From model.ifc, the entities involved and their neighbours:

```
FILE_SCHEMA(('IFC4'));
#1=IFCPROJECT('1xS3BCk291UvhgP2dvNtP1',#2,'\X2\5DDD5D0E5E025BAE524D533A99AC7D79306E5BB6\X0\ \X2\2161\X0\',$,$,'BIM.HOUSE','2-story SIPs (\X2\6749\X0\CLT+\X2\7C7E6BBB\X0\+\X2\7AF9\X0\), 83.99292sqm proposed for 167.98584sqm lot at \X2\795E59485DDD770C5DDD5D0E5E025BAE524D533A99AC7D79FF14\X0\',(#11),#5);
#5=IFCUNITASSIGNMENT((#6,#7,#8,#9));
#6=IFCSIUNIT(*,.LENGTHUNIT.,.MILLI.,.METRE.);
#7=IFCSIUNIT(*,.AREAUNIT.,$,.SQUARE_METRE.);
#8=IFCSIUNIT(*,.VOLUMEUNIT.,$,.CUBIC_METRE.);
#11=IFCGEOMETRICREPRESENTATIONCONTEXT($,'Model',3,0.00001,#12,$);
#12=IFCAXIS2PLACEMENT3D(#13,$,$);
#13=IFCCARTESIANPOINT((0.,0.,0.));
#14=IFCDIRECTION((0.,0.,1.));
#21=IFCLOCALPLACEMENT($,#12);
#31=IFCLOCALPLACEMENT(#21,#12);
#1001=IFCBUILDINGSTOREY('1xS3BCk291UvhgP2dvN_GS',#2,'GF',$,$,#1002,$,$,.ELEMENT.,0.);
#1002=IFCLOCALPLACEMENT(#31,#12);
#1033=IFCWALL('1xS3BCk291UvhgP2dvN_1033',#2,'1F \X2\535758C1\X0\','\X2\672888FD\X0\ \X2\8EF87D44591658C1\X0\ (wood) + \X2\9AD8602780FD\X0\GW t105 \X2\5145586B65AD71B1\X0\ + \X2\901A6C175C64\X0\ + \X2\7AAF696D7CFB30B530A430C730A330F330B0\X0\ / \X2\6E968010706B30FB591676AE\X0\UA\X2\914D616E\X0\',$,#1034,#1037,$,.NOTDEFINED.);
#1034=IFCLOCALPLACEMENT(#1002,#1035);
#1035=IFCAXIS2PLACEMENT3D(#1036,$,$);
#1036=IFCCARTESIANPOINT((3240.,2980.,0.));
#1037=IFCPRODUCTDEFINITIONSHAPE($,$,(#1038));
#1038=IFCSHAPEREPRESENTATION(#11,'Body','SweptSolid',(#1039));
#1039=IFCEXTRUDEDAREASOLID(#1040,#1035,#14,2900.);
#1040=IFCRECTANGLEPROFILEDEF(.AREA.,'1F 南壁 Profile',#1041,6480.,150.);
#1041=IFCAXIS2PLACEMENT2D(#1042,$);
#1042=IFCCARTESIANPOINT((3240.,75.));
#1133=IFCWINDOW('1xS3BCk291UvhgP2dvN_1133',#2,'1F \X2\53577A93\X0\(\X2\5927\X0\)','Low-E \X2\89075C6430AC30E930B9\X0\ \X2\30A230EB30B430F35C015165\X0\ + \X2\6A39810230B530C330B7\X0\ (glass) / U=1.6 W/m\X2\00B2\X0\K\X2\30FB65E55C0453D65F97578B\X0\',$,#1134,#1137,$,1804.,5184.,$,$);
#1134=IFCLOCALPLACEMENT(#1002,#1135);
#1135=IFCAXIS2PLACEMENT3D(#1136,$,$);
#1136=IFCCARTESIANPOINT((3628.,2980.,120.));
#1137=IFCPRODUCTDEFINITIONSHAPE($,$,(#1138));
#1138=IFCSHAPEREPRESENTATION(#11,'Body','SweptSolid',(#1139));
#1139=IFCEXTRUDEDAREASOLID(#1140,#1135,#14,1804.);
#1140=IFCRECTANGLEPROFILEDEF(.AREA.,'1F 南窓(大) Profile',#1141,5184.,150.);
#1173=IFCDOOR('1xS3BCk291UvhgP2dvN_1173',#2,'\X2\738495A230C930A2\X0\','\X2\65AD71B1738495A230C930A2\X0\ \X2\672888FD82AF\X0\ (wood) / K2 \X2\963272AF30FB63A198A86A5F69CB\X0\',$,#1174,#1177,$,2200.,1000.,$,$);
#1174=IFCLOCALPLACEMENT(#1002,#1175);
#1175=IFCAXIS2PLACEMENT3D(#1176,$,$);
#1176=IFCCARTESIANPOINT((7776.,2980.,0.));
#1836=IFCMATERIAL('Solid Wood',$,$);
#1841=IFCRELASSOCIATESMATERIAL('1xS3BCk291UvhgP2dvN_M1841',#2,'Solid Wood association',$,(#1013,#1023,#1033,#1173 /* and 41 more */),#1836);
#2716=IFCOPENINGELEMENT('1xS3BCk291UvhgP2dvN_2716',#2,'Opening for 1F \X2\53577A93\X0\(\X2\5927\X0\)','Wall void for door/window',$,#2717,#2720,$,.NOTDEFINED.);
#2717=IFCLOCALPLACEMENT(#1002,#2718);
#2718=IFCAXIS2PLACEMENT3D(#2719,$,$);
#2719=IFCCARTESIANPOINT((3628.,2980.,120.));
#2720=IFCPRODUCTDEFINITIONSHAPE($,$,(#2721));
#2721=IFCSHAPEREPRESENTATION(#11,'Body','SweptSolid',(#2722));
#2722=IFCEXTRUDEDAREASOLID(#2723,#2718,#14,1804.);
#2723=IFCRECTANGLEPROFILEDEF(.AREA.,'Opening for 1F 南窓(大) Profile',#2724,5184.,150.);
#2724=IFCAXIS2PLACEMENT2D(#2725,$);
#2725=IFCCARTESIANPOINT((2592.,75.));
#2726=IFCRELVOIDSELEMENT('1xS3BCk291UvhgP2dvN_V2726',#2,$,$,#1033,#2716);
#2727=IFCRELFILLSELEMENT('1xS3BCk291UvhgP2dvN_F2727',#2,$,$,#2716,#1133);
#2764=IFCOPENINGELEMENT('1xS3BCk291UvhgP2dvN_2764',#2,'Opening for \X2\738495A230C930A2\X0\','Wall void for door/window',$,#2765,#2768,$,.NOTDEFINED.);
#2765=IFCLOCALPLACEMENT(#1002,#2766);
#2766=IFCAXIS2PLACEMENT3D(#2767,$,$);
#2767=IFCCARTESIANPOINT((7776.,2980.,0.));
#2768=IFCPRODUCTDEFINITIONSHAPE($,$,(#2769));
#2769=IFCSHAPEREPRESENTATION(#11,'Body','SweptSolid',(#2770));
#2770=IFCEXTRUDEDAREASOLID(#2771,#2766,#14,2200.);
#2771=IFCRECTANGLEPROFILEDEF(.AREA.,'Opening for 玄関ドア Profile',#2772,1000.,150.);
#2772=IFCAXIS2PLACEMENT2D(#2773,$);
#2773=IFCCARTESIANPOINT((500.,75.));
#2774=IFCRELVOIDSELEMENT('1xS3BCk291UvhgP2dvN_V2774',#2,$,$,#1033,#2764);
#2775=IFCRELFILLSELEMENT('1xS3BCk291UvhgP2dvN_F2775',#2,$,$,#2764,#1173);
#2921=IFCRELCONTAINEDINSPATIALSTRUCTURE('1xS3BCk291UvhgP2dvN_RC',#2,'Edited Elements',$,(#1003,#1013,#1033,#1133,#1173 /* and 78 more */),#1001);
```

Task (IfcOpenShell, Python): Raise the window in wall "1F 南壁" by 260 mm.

```python
import numpy as np
import ifcopenshell
import ifcopenshell.api.geometry
import ifcopenshell.util.placement
import ifcopenshell.util.unit

model = ifcopenshell.open("model.ifc")
unit_scale = ifcopenshell.util.unit.calculate_unit_scale(model)

window = model.by_guid("1xS3BCk291UvhgP2dvN_1133")
opening = window.FillsVoids[0].RelatingOpeningElement
dz = 260.0

shift = np.array([0.0, 0.0, dz])
# The window is not placed relative to its opening, so move both.
for product in (opening, window):
    matrix = ifcopenshell.util.placement.get_local_placement(product.ObjectPlacement)
    matrix[:3, 3] += shift
    ifcopenshell.api.geometry.edit_object_placement(model, product=product, matrix=matrix, is_si=False)

print(f"moved by {dz * unit_scale:+.3f} m")

model.write("model_v2.ifc")
```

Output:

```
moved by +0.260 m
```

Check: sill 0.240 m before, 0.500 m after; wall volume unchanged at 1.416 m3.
